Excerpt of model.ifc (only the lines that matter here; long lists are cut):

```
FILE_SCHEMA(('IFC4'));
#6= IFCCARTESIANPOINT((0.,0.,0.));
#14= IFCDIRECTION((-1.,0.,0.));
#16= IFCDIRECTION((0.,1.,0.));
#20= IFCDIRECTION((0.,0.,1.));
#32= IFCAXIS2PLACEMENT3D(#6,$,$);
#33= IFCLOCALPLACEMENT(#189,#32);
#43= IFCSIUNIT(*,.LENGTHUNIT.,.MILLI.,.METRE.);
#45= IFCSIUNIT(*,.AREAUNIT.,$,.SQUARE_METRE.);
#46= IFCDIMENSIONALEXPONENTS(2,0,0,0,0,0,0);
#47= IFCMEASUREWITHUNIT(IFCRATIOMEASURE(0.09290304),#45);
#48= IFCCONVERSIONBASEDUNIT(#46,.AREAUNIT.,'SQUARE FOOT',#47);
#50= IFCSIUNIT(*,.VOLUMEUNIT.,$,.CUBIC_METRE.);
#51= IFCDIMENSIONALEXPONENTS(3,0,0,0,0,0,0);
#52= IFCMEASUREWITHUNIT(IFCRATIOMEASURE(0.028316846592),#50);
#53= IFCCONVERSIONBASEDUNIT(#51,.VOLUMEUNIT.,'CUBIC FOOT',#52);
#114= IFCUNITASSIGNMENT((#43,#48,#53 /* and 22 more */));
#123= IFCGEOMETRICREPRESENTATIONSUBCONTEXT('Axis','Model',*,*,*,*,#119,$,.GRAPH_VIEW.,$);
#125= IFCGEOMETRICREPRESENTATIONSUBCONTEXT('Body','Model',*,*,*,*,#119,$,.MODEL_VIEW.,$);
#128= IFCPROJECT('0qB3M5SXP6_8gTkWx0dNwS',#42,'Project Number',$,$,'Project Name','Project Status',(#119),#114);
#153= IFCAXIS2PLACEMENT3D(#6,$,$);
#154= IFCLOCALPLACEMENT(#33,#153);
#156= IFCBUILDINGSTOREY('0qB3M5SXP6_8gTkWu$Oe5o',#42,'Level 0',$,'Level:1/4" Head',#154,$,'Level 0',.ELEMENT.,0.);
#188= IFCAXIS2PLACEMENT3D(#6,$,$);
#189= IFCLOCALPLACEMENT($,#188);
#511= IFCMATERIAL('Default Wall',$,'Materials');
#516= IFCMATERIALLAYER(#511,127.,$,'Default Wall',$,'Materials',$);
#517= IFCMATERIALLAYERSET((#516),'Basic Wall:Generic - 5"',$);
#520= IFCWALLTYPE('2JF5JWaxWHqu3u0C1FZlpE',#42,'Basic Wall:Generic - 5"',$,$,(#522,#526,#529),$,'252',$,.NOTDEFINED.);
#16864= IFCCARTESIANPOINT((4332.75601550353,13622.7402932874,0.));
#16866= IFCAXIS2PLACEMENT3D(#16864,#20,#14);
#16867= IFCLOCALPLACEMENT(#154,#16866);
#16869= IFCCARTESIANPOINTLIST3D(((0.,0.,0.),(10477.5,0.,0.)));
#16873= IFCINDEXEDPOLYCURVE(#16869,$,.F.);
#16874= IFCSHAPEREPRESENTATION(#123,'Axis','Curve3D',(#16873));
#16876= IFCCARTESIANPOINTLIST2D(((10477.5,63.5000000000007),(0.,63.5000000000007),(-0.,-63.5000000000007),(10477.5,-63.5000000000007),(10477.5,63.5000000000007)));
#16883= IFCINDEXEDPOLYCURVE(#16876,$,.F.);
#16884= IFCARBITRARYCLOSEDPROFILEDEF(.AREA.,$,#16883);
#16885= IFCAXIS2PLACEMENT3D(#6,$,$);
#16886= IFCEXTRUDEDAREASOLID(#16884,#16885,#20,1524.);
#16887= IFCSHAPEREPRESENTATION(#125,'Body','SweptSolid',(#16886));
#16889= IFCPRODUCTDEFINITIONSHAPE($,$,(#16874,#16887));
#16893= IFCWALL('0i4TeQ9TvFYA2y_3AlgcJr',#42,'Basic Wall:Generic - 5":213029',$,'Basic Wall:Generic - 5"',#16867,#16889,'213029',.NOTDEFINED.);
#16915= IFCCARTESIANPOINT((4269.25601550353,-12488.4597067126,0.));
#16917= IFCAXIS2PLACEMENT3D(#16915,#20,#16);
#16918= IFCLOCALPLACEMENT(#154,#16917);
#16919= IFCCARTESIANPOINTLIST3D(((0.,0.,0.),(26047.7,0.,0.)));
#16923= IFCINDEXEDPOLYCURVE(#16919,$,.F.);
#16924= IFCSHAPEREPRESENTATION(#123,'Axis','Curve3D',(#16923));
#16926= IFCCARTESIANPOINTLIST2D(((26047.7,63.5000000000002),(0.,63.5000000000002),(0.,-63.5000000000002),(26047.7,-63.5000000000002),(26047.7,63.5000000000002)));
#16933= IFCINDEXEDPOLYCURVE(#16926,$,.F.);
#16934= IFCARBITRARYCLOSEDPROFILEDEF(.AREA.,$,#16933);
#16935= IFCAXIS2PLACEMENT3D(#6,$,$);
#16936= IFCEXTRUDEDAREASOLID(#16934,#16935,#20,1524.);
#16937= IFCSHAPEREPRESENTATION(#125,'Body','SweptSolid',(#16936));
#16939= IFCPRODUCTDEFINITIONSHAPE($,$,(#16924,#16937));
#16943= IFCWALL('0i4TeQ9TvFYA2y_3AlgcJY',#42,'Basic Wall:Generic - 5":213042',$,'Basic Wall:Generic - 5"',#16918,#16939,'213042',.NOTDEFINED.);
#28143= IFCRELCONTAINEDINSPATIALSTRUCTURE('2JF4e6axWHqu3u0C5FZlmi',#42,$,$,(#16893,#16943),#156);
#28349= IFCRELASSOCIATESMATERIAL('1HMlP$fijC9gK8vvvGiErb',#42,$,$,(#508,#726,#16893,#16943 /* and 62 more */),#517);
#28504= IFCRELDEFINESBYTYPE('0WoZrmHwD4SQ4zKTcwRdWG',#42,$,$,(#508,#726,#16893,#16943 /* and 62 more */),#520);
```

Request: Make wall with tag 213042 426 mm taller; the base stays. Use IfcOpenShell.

```python
import ifcopenshell
import ifcopenshell.geom
import ifcopenshell.util.representation
import ifcopenshell.util.shape
import ifcopenshell.util.unit

model = ifcopenshell.open("model.ifc")
unit_scale = ifcopenshell.util.unit.calculate_unit_scale(model)
settings = ifcopenshell.geom.settings()


def volume(element):
    """Net volume in cubic metres, openings subtracted."""
    shape = ifcopenshell.geom.create_shape(settings, element)
    return ifcopenshell.util.shape.get_volume(shape.geometry)


wall = model.by_guid("0i4TeQ9TvFYA2y_3AlgcJY")
before = volume(wall)

body = ifcopenshell.util.representation.get_representation(wall, "Model", "Body")
solid = body.Items[0]
old_height = solid.Depth
solid.Depth += 0.426 / unit_scale
after = volume(wall)

print(f"height {old_height:g} -> {solid.Depth:g}, volume {before:.3f} -> {after:.3f} m3")

model.write("model_rev.ifc")
```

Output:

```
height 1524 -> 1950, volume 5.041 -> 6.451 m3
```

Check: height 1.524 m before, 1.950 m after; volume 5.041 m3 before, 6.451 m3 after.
